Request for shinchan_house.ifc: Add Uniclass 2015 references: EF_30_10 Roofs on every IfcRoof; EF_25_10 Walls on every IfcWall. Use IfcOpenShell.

First a look at what the model holds.

```python
import ifcopenshell

model = ifcopenshell.open("shinchan_house.ifc")
print(model.schema)
print("classifications:", [c.Name for c in model.by_type("IfcClassification")])
for ifc_class in ("IfcDoor", "IfcRoof", "IfcStair", "IfcWall", "IfcWindow"):
    print(ifc_class, len(model.by_type(ifc_class)))
```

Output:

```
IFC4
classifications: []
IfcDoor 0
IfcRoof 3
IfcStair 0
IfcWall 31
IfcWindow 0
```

```python
import ifcopenshell
import ifcopenshell.api.classification

model = ifcopenshell.open("shinchan_house.ifc")

system = ifcopenshell.api.classification.add_classification(model, classification="Uniclass 2015")

codes = {
    "IfcRoof": ("EF_30_10", "Roofs"),
    "IfcWall": ("EF_25_10", "Walls"),
}
for ifc_class, (code, name) in codes.items():
    products = model.by_type(ifc_class)
    ifcopenshell.api.classification.add_reference(
        model, products=products, classification=system, identification=code, name=name
    )
    print(code, len(products))

model.write("shinchan_house_v2.ifc")
```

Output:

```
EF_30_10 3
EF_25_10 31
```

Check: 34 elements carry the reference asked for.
